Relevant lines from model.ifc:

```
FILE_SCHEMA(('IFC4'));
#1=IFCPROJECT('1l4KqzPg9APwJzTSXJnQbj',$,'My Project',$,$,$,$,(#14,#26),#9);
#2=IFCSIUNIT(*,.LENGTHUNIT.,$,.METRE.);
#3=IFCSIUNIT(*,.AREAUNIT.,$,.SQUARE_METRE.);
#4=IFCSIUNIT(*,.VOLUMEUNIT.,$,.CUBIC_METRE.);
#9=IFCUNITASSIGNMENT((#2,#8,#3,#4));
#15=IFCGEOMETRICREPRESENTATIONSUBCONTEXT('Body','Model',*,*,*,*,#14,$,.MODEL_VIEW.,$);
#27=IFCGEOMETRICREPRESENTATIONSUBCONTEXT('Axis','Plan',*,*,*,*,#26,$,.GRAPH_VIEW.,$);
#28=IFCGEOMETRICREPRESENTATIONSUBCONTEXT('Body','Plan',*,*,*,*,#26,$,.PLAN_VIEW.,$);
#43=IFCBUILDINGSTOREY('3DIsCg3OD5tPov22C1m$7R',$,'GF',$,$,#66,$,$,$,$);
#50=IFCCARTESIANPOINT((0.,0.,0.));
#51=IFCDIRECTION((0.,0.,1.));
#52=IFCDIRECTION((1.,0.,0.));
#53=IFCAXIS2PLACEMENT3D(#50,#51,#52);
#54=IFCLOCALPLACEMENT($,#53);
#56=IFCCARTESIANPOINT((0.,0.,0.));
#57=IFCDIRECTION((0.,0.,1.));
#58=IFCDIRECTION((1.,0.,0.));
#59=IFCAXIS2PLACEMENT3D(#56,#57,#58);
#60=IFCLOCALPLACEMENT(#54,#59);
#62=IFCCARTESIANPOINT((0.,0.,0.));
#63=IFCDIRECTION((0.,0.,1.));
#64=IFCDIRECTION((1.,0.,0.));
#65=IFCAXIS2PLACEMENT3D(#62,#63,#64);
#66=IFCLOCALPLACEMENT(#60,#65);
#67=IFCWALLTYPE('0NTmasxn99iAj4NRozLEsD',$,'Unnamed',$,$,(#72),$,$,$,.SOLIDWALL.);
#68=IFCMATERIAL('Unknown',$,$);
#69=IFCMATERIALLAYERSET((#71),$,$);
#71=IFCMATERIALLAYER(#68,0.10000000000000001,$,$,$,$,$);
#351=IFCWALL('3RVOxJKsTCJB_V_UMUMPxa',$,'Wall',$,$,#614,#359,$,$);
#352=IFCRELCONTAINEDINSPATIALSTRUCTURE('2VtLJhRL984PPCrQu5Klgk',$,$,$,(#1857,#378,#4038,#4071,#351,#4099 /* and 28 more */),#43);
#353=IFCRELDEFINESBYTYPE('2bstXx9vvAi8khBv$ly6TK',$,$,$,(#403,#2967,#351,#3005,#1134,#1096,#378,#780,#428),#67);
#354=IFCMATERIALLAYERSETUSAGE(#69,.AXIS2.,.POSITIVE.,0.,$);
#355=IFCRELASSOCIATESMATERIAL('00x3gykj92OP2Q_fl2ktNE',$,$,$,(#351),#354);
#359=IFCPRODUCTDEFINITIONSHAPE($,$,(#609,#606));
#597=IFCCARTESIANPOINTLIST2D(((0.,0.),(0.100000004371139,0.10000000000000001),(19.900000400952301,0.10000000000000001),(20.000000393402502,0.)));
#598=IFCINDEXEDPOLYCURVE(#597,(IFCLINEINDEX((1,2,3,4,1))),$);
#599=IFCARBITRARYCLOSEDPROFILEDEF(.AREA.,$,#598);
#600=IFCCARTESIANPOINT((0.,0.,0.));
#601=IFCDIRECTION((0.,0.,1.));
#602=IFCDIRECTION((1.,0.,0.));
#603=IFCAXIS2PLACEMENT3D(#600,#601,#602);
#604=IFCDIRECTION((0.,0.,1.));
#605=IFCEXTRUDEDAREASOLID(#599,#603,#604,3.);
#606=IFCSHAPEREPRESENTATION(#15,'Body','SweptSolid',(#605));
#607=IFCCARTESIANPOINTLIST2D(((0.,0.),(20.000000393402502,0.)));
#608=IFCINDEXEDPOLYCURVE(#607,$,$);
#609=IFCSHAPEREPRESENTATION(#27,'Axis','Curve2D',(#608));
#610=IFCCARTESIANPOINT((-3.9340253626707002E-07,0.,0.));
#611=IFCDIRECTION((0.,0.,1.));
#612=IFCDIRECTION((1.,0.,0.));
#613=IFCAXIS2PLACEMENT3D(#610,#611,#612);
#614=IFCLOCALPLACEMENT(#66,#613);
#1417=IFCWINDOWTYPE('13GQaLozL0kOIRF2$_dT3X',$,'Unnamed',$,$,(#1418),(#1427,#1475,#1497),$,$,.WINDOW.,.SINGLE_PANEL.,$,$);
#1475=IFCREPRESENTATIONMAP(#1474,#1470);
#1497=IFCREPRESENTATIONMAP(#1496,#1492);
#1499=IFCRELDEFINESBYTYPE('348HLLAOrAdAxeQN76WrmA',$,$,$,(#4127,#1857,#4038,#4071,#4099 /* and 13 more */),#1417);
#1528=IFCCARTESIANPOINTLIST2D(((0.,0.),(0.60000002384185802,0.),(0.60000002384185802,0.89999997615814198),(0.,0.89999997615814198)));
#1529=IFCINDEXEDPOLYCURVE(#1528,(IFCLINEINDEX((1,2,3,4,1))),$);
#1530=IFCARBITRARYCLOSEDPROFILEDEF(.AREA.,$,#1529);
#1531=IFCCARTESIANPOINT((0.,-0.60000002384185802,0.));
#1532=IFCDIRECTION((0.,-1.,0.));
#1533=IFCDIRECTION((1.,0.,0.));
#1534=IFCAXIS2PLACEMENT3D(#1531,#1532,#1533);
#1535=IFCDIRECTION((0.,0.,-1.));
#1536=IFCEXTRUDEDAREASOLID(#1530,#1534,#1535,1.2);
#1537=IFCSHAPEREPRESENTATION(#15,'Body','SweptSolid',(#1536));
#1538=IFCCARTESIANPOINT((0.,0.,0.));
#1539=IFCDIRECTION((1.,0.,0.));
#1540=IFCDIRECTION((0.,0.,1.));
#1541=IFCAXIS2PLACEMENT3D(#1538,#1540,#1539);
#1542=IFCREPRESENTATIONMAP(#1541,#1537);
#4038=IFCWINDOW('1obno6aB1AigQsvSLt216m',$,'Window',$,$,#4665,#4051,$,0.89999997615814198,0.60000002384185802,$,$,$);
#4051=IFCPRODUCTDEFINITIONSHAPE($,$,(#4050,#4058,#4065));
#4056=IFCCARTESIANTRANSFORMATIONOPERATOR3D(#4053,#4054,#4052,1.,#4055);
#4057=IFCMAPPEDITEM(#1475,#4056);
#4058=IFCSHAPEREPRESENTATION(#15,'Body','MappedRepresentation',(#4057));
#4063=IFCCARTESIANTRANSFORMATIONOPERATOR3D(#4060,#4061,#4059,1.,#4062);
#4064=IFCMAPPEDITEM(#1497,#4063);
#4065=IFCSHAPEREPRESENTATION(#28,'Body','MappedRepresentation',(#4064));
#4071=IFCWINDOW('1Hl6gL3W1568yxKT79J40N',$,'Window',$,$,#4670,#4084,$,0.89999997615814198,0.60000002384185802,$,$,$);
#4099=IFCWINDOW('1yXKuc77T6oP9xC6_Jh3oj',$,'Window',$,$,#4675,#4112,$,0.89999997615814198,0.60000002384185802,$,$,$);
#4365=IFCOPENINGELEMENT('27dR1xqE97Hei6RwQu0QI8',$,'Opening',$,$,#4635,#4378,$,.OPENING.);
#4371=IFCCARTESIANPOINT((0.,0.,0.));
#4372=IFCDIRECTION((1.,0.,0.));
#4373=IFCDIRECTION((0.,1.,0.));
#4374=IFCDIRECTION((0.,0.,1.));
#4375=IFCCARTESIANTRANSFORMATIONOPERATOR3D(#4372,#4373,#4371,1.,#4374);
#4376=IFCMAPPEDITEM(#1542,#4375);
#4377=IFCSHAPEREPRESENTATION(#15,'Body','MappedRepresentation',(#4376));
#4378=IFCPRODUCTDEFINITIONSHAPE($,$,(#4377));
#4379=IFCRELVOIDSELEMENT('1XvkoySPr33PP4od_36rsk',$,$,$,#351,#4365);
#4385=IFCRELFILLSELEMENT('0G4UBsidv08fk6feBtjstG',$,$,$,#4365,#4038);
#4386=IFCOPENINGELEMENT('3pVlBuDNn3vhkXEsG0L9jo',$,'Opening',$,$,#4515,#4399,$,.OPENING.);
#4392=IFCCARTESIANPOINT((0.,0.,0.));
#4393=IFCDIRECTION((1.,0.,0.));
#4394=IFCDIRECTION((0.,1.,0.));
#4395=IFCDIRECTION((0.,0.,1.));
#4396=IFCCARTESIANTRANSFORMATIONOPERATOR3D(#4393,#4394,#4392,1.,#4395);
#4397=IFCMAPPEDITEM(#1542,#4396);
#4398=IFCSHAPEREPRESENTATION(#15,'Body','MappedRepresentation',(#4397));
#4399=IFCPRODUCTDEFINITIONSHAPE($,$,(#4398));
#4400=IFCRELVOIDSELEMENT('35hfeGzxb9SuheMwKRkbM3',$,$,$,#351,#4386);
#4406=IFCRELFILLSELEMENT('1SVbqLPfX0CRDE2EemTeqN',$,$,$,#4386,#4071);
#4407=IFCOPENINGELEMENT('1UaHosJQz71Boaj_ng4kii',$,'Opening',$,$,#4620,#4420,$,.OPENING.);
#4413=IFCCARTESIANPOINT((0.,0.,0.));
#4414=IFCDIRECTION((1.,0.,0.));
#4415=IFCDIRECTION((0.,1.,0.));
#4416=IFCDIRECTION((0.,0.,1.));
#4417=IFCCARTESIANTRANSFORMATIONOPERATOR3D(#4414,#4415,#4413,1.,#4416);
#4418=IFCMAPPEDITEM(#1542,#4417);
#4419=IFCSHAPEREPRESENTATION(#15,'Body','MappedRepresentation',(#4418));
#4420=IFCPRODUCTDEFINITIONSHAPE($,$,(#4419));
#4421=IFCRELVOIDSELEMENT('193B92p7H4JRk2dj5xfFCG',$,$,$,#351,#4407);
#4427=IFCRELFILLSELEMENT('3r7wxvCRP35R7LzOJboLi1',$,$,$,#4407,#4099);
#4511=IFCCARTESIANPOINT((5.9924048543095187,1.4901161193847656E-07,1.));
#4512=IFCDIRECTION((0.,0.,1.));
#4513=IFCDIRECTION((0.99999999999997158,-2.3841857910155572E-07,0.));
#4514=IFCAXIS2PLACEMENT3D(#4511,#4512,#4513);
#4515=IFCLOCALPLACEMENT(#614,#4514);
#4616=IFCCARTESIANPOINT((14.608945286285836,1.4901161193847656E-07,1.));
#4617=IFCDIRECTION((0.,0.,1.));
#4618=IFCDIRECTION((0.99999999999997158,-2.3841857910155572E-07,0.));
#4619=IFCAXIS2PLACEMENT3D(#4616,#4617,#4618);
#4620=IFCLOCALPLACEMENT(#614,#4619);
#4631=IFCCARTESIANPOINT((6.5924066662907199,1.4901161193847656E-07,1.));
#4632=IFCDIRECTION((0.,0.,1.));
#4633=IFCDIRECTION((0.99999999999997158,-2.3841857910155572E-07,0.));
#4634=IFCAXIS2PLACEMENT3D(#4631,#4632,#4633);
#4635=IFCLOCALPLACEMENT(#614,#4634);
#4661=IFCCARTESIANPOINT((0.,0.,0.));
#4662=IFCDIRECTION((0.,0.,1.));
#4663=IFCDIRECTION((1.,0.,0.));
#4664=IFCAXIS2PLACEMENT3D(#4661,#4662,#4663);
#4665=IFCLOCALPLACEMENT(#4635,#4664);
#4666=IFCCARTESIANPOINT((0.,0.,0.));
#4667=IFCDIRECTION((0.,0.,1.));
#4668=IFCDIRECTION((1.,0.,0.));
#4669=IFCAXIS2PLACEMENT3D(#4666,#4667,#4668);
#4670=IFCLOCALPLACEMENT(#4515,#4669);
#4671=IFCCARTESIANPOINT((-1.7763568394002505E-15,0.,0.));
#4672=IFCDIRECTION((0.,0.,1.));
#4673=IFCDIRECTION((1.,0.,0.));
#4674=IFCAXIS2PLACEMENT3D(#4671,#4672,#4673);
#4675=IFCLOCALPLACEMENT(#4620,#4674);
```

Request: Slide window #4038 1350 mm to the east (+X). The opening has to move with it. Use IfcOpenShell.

```python
import ifcopenshell
import ifcopenshell.api.geometry
import ifcopenshell.util.placement

model = ifcopenshell.open("model.ifc")

window = model.by_id(4038)
opening = window.FillsVoids[0].RelatingOpeningElement
wall = opening.VoidsElements[0].RelatingBuildingElement

wall_matrix = ifcopenshell.util.placement.get_local_placement(wall.ObjectPlacement)
shift = wall_matrix[:3, 0] * 1.35
before = ifcopenshell.util.placement.get_local_placement(window.ObjectPlacement)[:3, 3].copy()

# The window is placed relative to its opening, so it follows when the opening moves.
matrix = ifcopenshell.util.placement.get_local_placement(opening.ObjectPlacement)
matrix[:3, 3] += shift
ifcopenshell.api.geometry.edit_object_placement(
    model, product=opening, matrix=matrix, is_si=False, should_transform_children=True
)

after = ifcopenshell.util.placement.get_local_placement(window.ObjectPlacement)[:3, 3]
print("window moved by", (after - before).round(3) + 0.0)

model.write("model_edited.ifc")
```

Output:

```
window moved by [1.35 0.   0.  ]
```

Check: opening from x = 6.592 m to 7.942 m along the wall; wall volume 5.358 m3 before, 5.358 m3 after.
